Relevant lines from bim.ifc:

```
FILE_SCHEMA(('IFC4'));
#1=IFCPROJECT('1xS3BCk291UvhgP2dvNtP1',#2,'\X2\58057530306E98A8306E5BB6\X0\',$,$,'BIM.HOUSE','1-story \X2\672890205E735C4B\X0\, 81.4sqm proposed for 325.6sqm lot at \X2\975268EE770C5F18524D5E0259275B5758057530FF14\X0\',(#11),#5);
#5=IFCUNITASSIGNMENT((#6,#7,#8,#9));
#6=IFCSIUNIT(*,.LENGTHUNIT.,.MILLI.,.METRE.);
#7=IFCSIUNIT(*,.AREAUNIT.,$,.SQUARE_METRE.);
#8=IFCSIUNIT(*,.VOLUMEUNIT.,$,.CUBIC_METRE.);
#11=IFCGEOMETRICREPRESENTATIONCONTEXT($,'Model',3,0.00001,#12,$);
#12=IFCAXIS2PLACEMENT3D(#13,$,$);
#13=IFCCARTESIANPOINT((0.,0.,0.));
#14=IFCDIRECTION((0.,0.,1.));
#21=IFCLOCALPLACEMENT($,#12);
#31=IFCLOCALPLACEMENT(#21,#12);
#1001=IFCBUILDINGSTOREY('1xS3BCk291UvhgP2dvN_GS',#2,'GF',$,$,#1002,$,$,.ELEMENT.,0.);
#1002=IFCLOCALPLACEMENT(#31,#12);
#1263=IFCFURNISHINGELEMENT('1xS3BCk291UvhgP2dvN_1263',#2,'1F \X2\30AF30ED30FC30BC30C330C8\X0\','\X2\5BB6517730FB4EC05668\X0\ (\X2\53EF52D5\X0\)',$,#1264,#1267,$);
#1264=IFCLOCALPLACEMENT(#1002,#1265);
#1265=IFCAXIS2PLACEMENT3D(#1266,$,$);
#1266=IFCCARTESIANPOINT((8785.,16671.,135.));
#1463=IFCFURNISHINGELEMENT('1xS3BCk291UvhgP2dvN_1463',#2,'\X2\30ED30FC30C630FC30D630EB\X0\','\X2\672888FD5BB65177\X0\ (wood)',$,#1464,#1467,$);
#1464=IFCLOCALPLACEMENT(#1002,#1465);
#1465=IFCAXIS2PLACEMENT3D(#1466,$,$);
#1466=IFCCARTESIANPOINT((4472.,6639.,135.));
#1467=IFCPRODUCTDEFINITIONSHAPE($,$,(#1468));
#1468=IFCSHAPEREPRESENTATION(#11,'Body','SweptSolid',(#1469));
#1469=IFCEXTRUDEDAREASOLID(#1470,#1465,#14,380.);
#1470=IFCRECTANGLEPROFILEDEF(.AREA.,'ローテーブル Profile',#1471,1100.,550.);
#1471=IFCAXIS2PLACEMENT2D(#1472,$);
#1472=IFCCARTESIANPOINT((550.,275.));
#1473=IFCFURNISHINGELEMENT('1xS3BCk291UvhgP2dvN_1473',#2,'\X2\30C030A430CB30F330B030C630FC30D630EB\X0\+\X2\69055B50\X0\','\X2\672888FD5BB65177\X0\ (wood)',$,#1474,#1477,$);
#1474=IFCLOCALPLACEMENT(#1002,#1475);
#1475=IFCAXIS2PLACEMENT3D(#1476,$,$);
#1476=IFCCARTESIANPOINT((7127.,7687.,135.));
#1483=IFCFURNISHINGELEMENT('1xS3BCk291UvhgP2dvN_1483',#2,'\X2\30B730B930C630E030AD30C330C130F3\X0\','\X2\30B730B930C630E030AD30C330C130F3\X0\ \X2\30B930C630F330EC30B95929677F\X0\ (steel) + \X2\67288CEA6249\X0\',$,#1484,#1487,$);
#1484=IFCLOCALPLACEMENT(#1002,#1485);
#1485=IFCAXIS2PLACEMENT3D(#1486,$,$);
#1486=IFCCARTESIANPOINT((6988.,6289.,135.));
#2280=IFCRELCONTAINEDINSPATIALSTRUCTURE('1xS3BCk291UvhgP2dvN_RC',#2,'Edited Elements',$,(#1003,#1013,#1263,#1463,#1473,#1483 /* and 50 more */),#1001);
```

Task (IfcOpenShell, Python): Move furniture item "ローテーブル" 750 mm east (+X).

```python
import ifcopenshell
import ifcopenshell.api.geometry
import ifcopenshell.util.placement
import ifcopenshell.util.unit

model = ifcopenshell.open("bim.ifc")
unit_scale = ifcopenshell.util.unit.calculate_unit_scale(model)

item = model.by_id(1463)
matrix = ifcopenshell.util.placement.get_local_placement(item.ObjectPlacement)
matrix[0, 3] += 0.75 / unit_scale
ifcopenshell.api.geometry.edit_object_placement(model, product=item, matrix=matrix, is_si=False)

print(ifcopenshell.util.placement.get_local_placement(item.ObjectPlacement).round(3) + 0.0)

model.write("bim_updated.ifc")
```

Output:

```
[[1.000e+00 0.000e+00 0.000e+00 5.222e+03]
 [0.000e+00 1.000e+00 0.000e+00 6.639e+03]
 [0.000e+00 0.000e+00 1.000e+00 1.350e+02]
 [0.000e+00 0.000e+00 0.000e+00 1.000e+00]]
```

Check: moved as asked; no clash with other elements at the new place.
